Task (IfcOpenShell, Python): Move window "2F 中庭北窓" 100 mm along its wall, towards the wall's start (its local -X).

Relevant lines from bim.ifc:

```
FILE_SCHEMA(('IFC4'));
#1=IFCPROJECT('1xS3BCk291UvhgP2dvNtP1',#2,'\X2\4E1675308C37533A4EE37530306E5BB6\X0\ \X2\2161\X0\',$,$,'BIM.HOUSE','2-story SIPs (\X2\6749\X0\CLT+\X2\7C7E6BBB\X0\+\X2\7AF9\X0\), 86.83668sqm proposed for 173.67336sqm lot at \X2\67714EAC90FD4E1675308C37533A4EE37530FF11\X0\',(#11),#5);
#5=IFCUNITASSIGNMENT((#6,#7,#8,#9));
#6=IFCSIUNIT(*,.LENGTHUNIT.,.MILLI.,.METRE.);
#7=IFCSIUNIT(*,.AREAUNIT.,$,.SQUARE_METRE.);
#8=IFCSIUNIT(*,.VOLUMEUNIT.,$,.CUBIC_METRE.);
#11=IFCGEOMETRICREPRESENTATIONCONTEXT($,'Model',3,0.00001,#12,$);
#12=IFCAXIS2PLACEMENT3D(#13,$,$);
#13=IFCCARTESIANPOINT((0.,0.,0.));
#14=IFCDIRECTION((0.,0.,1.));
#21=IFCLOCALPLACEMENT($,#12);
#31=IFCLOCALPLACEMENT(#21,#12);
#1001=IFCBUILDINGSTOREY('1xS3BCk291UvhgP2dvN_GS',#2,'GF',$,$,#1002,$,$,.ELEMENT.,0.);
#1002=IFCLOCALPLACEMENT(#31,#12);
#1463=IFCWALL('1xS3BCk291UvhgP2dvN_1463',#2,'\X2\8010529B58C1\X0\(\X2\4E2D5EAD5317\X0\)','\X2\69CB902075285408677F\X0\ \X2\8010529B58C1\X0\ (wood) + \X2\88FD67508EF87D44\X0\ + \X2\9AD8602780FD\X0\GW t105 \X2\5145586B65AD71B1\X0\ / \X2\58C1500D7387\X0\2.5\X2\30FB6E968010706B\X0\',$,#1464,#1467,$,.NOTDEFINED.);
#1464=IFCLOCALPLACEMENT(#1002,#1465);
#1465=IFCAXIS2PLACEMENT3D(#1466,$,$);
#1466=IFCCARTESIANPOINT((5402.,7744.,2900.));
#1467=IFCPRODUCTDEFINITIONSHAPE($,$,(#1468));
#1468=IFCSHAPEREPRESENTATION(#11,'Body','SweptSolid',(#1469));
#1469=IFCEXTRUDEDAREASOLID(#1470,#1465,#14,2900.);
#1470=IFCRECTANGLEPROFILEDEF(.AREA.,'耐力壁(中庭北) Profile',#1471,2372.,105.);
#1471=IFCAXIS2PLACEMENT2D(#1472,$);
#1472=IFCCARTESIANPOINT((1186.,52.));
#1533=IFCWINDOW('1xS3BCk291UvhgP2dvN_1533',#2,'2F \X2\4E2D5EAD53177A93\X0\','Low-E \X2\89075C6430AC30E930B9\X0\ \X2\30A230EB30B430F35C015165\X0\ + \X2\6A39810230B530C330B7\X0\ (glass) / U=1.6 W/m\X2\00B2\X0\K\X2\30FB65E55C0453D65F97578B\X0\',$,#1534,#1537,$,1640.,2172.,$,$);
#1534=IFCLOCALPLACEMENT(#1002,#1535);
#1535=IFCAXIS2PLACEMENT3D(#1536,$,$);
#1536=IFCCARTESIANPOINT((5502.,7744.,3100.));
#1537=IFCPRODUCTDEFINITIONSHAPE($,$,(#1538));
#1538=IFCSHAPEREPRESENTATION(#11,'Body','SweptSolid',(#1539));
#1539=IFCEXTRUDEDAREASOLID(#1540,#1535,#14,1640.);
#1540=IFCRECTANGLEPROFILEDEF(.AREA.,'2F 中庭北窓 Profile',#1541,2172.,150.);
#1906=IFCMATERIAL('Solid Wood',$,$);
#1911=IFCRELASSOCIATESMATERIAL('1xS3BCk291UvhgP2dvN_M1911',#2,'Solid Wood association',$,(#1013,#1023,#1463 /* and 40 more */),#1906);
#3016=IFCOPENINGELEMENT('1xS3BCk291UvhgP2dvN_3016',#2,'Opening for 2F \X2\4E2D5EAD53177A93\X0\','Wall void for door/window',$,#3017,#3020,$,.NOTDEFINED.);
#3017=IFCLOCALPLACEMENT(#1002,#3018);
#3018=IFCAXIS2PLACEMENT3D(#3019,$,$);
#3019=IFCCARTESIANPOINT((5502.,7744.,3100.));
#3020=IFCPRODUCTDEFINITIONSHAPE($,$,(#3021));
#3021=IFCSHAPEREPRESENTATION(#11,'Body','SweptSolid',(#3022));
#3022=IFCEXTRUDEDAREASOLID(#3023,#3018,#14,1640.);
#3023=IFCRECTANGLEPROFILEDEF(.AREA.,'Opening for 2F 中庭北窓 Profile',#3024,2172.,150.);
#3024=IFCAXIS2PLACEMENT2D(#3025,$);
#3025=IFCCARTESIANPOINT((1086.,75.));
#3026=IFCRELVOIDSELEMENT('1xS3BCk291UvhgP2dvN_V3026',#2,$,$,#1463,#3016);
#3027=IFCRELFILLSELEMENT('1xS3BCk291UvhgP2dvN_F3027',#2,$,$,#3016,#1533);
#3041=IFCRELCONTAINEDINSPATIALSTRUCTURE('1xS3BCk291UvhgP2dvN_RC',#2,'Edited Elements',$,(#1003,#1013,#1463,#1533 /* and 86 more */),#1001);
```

```python
import ifcopenshell
import ifcopenshell.api.geometry
import ifcopenshell.util.placement

model = ifcopenshell.open("bim.ifc")

window = model.by_guid("1xS3BCk291UvhgP2dvN_1533")
opening = window.FillsVoids[0].RelatingOpeningElement
wall = opening.VoidsElements[0].RelatingBuildingElement

wall_matrix = ifcopenshell.util.placement.get_local_placement(wall.ObjectPlacement)
shift = wall_matrix[:3, 0] * -100.0
before = ifcopenshell.util.placement.get_local_placement(window.ObjectPlacement)[:3, 3].copy()

# The window is not placed relative to its opening, so move both.
for product in (opening, window):
    matrix = ifcopenshell.util.placement.get_local_placement(product.ObjectPlacement)
    matrix[:3, 3] += shift
    ifcopenshell.api.geometry.edit_object_placement(model, product=product, matrix=matrix, is_si=False)

after = ifcopenshell.util.placement.get_local_placement(window.ObjectPlacement)[:3, 3]
print("window moved by", (after - before).round(3) + 0.0)

model.write("bim_updated.ifc")
```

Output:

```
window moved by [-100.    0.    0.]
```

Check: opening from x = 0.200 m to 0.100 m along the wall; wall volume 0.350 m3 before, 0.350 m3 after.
